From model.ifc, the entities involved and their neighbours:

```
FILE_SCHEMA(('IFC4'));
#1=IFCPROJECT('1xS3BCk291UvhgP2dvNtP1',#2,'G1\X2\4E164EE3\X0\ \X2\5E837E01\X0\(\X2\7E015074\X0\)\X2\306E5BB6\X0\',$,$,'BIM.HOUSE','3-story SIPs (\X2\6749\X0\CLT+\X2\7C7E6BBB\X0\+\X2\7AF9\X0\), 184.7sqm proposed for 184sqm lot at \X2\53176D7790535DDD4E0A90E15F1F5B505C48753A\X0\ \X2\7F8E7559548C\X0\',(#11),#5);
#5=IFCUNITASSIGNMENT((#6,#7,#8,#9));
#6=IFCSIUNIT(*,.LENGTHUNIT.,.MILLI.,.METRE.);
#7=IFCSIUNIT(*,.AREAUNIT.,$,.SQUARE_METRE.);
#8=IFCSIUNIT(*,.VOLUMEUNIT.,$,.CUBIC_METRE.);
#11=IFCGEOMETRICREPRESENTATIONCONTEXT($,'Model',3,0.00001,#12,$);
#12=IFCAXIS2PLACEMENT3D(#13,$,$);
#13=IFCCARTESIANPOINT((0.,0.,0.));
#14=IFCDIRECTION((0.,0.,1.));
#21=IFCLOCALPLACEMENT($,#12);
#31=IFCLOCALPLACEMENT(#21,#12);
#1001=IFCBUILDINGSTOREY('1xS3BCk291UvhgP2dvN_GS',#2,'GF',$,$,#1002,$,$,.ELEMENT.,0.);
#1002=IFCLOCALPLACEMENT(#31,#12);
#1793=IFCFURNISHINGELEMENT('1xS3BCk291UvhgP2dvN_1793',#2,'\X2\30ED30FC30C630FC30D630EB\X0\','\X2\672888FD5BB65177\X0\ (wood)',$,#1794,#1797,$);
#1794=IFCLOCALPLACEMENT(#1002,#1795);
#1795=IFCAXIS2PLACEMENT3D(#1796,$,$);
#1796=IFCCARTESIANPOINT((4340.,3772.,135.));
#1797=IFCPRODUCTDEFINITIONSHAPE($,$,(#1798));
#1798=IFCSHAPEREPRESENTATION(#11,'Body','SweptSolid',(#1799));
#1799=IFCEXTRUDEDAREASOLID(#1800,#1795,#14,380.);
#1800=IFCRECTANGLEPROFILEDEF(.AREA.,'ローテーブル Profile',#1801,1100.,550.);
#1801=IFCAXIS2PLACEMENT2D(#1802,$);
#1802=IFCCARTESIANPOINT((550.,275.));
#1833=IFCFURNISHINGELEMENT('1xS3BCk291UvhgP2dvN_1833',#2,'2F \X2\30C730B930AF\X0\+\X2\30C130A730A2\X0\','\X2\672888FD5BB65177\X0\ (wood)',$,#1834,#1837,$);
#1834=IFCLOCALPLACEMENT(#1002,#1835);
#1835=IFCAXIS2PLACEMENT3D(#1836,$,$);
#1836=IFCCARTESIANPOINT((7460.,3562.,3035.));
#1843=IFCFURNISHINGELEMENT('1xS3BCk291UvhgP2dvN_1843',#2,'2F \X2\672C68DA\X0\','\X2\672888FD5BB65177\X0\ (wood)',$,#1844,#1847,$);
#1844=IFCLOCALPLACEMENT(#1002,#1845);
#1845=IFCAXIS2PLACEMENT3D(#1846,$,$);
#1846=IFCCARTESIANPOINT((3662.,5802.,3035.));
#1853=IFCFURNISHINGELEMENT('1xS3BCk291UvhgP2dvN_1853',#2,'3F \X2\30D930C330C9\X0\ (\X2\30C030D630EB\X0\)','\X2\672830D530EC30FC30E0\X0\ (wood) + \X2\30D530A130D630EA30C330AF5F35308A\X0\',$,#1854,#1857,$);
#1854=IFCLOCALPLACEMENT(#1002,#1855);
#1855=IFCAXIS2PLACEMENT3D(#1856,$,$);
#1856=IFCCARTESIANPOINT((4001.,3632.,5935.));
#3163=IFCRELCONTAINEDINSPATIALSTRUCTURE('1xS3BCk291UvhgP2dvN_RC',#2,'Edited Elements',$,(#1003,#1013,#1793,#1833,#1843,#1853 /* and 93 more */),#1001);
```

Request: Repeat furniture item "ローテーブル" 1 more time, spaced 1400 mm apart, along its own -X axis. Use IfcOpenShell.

```python
import ifcopenshell
import ifcopenshell.api.geometry
import ifcopenshell.api.root
import ifcopenshell.util.element
import ifcopenshell.util.placement

model = ifcopenshell.open("model.ifc")


def reuse_history(source, copy):
    """copy_class also copies each property set's owner history, people and application; keep the originals."""
    for rel in copy.IsDefinedBy:
        if rel.is_a("IfcRelDefinesByProperties") and (history := rel.RelatingPropertyDefinition.OwnerHistory):
            rel.RelatingPropertyDefinition.OwnerHistory = source.OwnerHistory
            ifcopenshell.util.element.remove_deep2(model, history)


source = model.by_id(1793)
base = ifcopenshell.util.placement.get_local_placement(source.ObjectPlacement)
step = -base[:3, 0] * 1400.0

for i in range(1, 2):
    copy = ifcopenshell.api.root.copy_class(model, product=source)
    copy.Representation = ifcopenshell.util.element.copy_deep(
        model, source.Representation, exclude=["IfcGeometricRepresentationContext", "IfcRepresentationMap"]
    )
    reuse_history(source, copy)
    matrix = base.copy()
    matrix[:3, 3] += i * step
    print("added at", matrix[:3, 3].round(3) + 0.0)
    ifcopenshell.api.geometry.edit_object_placement(model, product=copy, matrix=matrix, is_si=False)

model.write("model_updated.ifc")
```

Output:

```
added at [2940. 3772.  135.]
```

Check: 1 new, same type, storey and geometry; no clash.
